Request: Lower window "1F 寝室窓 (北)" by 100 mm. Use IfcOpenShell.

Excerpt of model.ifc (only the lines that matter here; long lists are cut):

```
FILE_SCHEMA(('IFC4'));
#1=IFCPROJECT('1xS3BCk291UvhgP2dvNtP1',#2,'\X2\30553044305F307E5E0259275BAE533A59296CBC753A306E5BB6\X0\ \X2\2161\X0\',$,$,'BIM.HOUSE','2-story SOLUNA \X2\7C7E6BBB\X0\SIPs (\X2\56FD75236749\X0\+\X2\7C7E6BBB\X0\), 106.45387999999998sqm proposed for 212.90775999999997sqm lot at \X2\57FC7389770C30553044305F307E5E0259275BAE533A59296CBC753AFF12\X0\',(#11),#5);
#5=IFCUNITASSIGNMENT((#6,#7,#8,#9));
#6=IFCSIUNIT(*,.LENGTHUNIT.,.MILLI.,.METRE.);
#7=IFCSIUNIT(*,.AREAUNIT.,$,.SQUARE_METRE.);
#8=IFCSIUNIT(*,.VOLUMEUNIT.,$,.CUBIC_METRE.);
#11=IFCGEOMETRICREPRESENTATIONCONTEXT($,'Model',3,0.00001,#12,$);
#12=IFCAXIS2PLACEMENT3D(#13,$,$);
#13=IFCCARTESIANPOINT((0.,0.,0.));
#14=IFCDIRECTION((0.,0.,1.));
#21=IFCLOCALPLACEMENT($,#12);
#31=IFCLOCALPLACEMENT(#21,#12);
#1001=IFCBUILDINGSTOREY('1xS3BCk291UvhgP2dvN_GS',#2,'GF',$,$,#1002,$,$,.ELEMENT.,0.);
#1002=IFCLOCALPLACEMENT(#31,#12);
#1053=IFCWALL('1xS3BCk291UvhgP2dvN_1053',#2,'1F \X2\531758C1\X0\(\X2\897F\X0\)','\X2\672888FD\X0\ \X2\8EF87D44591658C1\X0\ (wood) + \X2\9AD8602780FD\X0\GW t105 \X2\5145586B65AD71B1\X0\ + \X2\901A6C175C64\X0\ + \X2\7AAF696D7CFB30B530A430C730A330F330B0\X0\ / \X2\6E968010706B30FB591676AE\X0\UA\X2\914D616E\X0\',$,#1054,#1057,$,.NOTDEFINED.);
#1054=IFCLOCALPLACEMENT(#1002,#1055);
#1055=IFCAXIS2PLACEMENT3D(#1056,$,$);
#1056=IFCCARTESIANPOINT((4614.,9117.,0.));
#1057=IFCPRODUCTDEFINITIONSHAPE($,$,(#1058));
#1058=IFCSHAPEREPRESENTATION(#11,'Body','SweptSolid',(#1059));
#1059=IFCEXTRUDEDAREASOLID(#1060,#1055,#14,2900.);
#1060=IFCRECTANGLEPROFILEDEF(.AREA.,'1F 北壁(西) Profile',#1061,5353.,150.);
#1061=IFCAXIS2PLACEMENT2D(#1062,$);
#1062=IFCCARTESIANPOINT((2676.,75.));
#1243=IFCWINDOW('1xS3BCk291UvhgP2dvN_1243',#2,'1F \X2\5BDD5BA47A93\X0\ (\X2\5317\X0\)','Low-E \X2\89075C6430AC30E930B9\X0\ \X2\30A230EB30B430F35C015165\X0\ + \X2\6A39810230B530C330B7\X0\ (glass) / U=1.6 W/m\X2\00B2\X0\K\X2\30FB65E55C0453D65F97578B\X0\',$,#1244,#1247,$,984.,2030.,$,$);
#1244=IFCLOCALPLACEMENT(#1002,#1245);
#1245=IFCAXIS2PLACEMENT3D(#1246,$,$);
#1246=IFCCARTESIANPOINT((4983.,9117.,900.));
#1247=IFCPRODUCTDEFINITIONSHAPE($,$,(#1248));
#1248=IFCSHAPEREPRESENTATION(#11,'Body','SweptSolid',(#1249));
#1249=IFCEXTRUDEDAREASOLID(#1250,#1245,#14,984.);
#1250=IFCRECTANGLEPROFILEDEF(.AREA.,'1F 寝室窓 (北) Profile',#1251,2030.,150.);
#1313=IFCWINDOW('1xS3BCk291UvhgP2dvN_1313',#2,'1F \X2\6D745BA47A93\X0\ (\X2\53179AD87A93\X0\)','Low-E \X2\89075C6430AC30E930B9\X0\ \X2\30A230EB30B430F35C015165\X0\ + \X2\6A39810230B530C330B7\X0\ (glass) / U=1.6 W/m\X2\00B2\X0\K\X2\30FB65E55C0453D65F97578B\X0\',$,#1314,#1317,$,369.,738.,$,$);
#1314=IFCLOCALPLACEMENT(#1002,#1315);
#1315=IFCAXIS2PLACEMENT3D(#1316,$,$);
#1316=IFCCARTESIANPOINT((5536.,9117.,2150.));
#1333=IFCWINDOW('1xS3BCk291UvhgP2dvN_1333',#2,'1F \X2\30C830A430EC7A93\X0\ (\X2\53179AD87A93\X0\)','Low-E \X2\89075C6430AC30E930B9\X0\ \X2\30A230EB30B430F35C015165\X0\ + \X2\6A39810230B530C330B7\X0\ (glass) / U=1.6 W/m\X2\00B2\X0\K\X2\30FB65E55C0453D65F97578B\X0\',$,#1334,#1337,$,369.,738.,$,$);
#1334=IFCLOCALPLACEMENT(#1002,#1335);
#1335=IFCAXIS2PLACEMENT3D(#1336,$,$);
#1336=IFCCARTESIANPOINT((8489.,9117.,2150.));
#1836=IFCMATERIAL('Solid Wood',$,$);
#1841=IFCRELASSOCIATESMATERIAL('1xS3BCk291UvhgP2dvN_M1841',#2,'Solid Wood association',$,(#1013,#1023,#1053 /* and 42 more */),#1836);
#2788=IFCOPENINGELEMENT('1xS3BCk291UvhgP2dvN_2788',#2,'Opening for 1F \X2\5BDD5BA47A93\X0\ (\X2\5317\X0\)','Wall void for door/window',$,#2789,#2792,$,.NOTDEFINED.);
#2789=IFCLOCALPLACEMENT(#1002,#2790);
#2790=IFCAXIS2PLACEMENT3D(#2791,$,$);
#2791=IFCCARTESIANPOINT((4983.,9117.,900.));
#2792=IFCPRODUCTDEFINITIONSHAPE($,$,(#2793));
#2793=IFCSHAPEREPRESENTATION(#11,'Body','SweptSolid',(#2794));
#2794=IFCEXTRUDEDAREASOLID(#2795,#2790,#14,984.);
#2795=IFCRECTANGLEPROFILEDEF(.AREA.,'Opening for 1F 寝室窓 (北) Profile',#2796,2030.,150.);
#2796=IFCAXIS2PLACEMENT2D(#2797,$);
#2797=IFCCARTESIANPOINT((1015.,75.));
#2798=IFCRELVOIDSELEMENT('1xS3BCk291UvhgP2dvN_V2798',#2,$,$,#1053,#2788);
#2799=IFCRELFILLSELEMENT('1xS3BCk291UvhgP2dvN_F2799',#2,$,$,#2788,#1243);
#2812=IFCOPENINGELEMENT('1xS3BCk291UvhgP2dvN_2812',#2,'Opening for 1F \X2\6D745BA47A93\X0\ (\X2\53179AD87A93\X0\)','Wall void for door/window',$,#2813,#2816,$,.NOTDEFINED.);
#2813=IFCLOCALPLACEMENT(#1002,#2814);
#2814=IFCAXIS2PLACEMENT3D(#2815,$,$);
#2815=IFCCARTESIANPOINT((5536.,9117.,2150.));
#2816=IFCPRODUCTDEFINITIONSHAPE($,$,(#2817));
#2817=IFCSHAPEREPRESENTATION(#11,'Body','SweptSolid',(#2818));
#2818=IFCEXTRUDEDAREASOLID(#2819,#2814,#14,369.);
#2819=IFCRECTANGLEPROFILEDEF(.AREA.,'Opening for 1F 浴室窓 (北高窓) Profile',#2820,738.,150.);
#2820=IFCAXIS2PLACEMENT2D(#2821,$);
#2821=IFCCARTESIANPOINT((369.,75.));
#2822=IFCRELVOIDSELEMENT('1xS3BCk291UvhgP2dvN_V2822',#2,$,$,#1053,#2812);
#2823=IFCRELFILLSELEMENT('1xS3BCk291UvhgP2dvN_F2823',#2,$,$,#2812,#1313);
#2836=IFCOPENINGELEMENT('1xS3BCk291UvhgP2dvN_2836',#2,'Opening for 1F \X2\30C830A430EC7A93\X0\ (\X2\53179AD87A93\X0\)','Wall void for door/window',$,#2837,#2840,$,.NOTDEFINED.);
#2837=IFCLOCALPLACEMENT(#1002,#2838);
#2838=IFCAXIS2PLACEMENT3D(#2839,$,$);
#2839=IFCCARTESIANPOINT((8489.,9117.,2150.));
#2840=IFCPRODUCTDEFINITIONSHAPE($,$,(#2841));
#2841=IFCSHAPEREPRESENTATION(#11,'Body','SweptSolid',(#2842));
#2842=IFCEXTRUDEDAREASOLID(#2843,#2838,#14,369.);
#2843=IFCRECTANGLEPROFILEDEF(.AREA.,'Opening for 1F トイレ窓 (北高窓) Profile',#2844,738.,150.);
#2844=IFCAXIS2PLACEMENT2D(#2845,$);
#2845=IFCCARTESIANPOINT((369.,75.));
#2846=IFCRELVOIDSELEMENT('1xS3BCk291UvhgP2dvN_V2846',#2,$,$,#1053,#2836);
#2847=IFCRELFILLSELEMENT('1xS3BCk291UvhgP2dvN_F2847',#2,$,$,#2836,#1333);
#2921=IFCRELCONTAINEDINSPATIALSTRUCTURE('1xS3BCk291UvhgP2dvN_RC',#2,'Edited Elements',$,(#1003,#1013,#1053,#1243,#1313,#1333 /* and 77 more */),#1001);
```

```python
import numpy as np
import ifcopenshell
import ifcopenshell.api.geometry
import ifcopenshell.util.placement
import ifcopenshell.util.unit

model = ifcopenshell.open("model.ifc")
unit_scale = ifcopenshell.util.unit.calculate_unit_scale(model)

window = model.by_id(1243)
opening = window.FillsVoids[0].RelatingOpeningElement
dz = -0.1 / unit_scale

shift = np.array([0.0, 0.0, dz])
# The window is not placed relative to its opening, so move both.
for product in (opening, window):
    matrix = ifcopenshell.util.placement.get_local_placement(product.ObjectPlacement)
    matrix[:3, 3] += shift
    ifcopenshell.api.geometry.edit_object_placement(model, product=product, matrix=matrix, is_si=False)

print(f"moved by {dz * unit_scale:+.3f} m")

model.write("model_updated.ifc")
```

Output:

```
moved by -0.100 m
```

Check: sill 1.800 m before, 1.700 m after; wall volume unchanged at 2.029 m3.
